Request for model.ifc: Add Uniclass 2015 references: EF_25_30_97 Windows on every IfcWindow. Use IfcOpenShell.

First a look at what the model holds.

```python
import ifcopenshell

model = ifcopenshell.open("model.ifc")
print(model.schema)
print("classifications:", [c.Name for c in model.by_type("IfcClassification")])
for ifc_class in ("IfcDoor", "IfcRoof", "IfcStair", "IfcWall", "IfcWindow"):
    print(ifc_class, len(model.by_type(ifc_class)))
```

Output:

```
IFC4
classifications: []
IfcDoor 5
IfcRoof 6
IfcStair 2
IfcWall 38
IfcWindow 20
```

```python
import ifcopenshell
import ifcopenshell.api.classification

model = ifcopenshell.open("model.ifc")

system = ifcopenshell.api.classification.add_classification(model, classification="Uniclass 2015")

codes = {
    "IfcWindow": ("EF_25_30_97", "Windows"),
}
for ifc_class, (code, name) in codes.items():
    products = model.by_type(ifc_class)
    ifcopenshell.api.classification.add_reference(
        model, products=products, classification=system, identification=code, name=name
    )
    print(code, len(products))

model.write("model_v2.ifc")
```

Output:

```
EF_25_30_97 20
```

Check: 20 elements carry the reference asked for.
